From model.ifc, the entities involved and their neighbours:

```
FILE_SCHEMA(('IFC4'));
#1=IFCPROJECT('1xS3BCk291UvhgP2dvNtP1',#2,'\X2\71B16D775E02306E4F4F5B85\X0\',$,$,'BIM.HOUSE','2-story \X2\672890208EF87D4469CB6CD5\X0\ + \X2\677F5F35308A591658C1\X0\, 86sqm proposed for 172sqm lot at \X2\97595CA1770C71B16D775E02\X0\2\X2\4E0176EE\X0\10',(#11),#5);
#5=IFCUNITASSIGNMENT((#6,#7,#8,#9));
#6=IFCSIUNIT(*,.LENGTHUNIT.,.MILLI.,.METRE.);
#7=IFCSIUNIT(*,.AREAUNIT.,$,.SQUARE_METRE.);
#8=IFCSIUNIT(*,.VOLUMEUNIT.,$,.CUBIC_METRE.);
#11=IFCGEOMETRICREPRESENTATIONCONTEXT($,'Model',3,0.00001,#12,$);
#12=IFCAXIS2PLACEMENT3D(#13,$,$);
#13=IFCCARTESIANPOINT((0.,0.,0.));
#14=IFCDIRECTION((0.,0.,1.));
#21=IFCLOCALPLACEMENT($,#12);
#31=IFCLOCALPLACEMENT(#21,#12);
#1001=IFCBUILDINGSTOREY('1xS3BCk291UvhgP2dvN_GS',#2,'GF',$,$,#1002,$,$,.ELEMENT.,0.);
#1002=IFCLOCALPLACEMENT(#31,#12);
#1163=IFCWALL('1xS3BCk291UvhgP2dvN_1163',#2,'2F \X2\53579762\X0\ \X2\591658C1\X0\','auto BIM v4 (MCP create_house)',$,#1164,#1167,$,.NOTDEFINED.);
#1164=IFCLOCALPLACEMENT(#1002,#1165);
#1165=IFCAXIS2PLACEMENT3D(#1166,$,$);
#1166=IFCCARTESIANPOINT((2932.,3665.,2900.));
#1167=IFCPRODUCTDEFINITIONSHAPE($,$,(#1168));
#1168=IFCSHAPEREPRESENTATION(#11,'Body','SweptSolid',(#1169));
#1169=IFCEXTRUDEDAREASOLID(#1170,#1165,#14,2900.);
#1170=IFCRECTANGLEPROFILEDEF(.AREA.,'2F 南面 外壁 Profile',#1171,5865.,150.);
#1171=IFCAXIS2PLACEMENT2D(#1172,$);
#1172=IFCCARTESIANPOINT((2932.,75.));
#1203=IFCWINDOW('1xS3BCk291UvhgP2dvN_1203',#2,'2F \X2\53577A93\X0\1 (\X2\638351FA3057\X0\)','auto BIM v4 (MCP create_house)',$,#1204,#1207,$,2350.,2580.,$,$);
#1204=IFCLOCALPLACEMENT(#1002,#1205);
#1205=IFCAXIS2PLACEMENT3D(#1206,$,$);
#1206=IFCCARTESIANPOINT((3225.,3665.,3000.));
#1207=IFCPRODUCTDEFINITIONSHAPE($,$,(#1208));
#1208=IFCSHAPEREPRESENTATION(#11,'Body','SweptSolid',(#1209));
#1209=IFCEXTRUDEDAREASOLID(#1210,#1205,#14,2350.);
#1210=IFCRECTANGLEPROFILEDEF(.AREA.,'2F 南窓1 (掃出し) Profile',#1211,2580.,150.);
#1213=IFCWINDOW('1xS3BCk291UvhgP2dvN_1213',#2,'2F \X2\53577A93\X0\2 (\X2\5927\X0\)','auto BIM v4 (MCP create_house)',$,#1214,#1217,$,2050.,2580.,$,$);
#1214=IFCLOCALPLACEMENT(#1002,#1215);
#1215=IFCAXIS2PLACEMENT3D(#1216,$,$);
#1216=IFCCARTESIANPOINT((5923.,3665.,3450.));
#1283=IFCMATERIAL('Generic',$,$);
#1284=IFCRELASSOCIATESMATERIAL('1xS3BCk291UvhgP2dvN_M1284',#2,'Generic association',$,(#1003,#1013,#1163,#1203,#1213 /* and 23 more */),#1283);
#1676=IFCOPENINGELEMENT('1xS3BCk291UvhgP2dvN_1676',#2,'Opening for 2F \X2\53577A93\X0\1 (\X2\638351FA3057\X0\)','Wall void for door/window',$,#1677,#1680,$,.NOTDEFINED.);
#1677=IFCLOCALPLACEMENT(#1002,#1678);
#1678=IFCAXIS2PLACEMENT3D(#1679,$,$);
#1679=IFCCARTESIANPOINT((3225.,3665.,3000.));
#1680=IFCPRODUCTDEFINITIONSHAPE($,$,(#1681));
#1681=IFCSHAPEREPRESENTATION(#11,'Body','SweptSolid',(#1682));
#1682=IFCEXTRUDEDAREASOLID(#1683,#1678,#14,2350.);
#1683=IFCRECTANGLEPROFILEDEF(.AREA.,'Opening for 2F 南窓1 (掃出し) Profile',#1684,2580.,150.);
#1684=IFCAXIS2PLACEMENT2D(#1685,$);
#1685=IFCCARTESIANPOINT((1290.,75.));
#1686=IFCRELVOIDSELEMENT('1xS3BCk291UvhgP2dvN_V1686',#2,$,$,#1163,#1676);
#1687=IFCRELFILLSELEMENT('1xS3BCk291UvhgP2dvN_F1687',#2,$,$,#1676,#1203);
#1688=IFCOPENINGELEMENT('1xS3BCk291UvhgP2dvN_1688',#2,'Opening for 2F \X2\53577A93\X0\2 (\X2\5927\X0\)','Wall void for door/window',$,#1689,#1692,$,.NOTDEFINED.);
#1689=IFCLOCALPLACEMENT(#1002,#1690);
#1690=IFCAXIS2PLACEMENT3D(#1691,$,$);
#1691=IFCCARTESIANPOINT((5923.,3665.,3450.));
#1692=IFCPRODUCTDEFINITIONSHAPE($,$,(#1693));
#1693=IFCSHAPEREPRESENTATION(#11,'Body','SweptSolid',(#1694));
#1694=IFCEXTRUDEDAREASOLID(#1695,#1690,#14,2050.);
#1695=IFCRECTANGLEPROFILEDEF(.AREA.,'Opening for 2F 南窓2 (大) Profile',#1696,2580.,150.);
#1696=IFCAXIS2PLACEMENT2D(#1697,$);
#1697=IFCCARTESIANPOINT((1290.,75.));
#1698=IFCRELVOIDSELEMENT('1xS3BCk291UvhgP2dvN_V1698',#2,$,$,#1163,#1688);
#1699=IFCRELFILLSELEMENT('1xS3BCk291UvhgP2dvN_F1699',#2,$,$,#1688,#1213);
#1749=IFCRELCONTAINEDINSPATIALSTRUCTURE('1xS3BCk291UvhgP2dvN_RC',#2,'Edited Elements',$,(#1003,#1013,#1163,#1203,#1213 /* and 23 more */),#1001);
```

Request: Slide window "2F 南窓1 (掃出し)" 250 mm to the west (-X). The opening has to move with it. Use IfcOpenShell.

```python
import ifcopenshell
import ifcopenshell.api.geometry
import ifcopenshell.util.placement

model = ifcopenshell.open("model.ifc")

window = model.by_id(1203)
opening = window.FillsVoids[0].RelatingOpeningElement
wall = opening.VoidsElements[0].RelatingBuildingElement

wall_matrix = ifcopenshell.util.placement.get_local_placement(wall.ObjectPlacement)
shift = wall_matrix[:3, 0] * -250.0
before = ifcopenshell.util.placement.get_local_placement(window.ObjectPlacement)[:3, 3].copy()

# The window is not placed relative to its opening, so move both.
for product in (opening, window):
    matrix = ifcopenshell.util.placement.get_local_placement(product.ObjectPlacement)
    matrix[:3, 3] += shift
    ifcopenshell.api.geometry.edit_object_placement(model, product=product, matrix=matrix, is_si=False)

after = ifcopenshell.util.placement.get_local_placement(window.ObjectPlacement)[:3, 3]
print("window moved by", (after - before).round(3) + 0.0)

model.write("model-out.ifc")
```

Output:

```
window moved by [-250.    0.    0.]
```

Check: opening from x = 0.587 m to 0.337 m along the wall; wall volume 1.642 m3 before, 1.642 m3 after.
